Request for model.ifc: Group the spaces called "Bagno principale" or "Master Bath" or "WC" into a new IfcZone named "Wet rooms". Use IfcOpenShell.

First a look at what the model holds.

```python
import ifcopenshell

model = ifcopenshell.open("model.ifc")
print(model.schema)
seen = {}
for space in model.by_type("IfcSpace"):
    seen[space.LongName] = seen.get(space.LongName, 0) + 1
for name, count in sorted(seen.items(), key=str):
    print(count, "x", name)
print("zones:", [z.Name for z in model.by_type("IfcZone")][:20])
```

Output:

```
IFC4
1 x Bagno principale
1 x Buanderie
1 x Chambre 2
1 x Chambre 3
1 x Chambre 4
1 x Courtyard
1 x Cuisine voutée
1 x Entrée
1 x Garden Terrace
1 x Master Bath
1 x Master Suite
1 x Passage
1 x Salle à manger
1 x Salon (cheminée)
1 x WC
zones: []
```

```python
import ifcopenshell
import ifcopenshell.api.group
import ifcopenshell.api.root

model = ifcopenshell.open("model.ifc")

names = {"Bagno principale", "Master Bath", "WC"}
spaces = [s for s in model.by_type("IfcSpace") if s.LongName in names]

zone = ifcopenshell.api.root.create_entity(model, ifc_class="IfcZone", name="Wet rooms")
ifcopenshell.api.group.assign_group(model, products=spaces, group=zone)
print(len(spaces), "spaces in", zone.Name)

model.write("model-out.ifc")
```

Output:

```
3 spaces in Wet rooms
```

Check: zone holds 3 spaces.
